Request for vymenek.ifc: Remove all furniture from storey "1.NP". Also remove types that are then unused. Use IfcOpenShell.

First a look at what the model holds.

```python
import ifcopenshell
import ifcopenshell.util.element

model = ifcopenshell.open("vymenek.ifc")
print(model.schema)
storey = next(s for s in model.by_type("IfcBuildingStorey") if s.Name == "1.NP")
furniture = [e for e in ifcopenshell.util.element.get_decomposition(storey) if e.is_a("IfcFurnishingElement")]
seen = {}
for e in furniture:
    element_type = ifcopenshell.util.element.get_type(e)
    name = element_type.Name if element_type not in (None, e) else None
    seen[name] = seen.get(name, 0) + 1
for name, count in sorted(seen.items(), key=str):
    print(count, "x", name)
```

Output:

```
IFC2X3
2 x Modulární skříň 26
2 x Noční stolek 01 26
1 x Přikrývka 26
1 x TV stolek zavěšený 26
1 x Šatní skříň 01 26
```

```python
import ifcopenshell
import ifcopenshell.api.root
import ifcopenshell.util.element

model = ifcopenshell.open("vymenek.ifc")

storey = next(s for s in model.by_type("IfcBuildingStorey") if s.Name == "1.NP")
furniture = [e for e in ifcopenshell.util.element.get_decomposition(storey) if e.is_a("IfcFurnishingElement")]
types = {ifcopenshell.util.element.get_type(e) for e in furniture} - {None, *furniture}

for e in furniture:
    ifcopenshell.api.root.remove_product(model, product=e)
print(len(furniture), "removed")

unused = [t for t in types if not ifcopenshell.util.element.get_types(t)]
for t in unused:
    ifcopenshell.api.root.remove_product(model, product=t)
print(len(unused), "unused types removed")

model.write("vymenek_edited.ifc")
```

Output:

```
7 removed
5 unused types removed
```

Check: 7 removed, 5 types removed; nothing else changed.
